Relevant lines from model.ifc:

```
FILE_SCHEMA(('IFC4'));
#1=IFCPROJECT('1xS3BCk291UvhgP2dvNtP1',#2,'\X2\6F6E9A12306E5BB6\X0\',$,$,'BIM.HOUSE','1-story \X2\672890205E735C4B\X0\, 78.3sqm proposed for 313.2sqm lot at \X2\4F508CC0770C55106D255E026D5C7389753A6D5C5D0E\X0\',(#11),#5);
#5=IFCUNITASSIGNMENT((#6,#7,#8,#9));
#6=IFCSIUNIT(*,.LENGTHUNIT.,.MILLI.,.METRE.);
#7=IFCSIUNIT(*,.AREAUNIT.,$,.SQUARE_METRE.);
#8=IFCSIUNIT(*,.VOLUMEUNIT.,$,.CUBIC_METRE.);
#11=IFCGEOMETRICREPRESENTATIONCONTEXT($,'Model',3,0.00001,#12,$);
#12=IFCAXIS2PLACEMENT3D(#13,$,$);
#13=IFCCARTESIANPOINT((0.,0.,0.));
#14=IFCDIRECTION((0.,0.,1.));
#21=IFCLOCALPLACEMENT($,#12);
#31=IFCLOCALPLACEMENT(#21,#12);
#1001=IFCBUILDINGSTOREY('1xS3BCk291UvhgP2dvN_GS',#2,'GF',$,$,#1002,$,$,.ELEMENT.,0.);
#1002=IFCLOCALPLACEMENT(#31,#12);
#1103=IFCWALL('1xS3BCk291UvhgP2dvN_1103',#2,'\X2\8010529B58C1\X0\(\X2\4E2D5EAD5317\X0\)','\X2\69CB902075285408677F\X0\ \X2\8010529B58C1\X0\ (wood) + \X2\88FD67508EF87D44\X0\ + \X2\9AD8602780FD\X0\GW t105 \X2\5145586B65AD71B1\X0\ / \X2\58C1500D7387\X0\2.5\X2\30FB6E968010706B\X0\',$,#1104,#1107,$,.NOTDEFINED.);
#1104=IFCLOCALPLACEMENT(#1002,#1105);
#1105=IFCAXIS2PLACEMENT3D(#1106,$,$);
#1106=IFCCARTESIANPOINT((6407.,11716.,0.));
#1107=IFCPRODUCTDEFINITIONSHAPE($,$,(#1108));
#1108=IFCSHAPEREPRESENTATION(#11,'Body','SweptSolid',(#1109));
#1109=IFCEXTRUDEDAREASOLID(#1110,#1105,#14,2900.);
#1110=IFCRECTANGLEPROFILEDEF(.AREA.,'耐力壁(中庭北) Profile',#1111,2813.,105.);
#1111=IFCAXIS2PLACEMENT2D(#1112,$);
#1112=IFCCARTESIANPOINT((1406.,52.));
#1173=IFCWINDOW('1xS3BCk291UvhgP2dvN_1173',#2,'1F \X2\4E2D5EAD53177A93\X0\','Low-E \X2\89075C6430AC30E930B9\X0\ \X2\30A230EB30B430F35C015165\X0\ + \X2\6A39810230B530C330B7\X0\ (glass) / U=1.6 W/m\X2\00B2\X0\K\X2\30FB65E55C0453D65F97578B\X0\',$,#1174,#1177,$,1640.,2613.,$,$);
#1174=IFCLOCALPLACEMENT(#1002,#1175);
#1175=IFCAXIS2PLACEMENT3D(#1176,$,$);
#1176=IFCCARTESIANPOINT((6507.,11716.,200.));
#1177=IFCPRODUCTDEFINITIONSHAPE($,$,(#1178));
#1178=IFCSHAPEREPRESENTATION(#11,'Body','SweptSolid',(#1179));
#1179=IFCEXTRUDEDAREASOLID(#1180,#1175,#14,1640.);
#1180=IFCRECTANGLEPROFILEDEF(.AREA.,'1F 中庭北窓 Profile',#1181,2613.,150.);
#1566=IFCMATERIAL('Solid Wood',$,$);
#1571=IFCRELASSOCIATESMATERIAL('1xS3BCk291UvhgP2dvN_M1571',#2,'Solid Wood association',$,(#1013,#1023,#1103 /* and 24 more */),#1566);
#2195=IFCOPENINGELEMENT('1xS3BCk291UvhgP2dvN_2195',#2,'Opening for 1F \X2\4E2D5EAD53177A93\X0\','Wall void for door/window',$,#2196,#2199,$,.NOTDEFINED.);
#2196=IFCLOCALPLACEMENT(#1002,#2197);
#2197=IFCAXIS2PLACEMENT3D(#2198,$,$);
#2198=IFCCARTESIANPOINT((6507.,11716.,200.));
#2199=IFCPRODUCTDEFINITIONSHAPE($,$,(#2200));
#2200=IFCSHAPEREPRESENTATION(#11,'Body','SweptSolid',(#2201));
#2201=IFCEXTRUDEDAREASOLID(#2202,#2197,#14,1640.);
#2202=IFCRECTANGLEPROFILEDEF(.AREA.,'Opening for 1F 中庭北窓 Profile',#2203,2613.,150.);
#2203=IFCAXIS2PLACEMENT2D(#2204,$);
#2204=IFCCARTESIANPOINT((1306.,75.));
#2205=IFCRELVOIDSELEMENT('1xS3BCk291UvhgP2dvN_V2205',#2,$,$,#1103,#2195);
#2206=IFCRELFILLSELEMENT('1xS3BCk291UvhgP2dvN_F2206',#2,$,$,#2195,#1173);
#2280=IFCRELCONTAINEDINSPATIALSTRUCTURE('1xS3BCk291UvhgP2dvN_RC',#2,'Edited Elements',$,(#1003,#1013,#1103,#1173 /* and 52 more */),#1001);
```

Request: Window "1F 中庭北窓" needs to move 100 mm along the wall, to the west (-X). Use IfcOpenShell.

```python
import ifcopenshell
import ifcopenshell.api.geometry
import ifcopenshell.util.placement

model = ifcopenshell.open("model.ifc")

window = model.by_guid("1xS3BCk291UvhgP2dvN_1173")
opening = window.FillsVoids[0].RelatingOpeningElement
wall = opening.VoidsElements[0].RelatingBuildingElement

wall_matrix = ifcopenshell.util.placement.get_local_placement(wall.ObjectPlacement)
shift = wall_matrix[:3, 0] * -100.0
before = ifcopenshell.util.placement.get_local_placement(window.ObjectPlacement)[:3, 3].copy()

# The window is not placed relative to its opening, so move both.
for product in (opening, window):
    matrix = ifcopenshell.util.placement.get_local_placement(product.ObjectPlacement)
    matrix[:3, 3] += shift
    ifcopenshell.api.geometry.edit_object_placement(model, product=product, matrix=matrix, is_si=False)

after = ifcopenshell.util.placement.get_local_placement(window.ObjectPlacement)[:3, 3]
print("window moved by", (after - before).round(3) + 0.0)

model.write("model_edited.ifc")
```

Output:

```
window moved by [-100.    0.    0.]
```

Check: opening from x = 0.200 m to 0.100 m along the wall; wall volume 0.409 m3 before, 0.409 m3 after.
